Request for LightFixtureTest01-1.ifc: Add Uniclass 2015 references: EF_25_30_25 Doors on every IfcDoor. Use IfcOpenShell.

First a look at what the model holds.

```python
import ifcopenshell

model = ifcopenshell.open("LightFixtureTest01-1.ifc")
print(model.schema)
print("classifications:", [c.Name for c in model.by_type("IfcClassification")])
for ifc_class in ("IfcDoor", "IfcRoof", "IfcStair", "IfcWall", "IfcWindow"):
    print(ifc_class, len(model.by_type(ifc_class)))
```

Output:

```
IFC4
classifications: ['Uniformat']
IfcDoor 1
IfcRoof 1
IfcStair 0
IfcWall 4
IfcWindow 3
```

```python
import ifcopenshell
import ifcopenshell.api.classification

model = ifcopenshell.open("LightFixtureTest01-1.ifc")

system = ifcopenshell.api.classification.add_classification(model, classification="Uniclass 2015")

codes = {
    "IfcDoor": ("EF_25_30_25", "Doors"),
}
for ifc_class, (code, name) in codes.items():
    products = model.by_type(ifc_class)
    ifcopenshell.api.classification.add_reference(
        model, products=products, classification=system, identification=code, name=name
    )
    print(code, len(products))

model.write("LightFixtureTest01-1_rev.ifc")
```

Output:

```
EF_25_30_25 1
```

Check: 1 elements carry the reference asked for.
